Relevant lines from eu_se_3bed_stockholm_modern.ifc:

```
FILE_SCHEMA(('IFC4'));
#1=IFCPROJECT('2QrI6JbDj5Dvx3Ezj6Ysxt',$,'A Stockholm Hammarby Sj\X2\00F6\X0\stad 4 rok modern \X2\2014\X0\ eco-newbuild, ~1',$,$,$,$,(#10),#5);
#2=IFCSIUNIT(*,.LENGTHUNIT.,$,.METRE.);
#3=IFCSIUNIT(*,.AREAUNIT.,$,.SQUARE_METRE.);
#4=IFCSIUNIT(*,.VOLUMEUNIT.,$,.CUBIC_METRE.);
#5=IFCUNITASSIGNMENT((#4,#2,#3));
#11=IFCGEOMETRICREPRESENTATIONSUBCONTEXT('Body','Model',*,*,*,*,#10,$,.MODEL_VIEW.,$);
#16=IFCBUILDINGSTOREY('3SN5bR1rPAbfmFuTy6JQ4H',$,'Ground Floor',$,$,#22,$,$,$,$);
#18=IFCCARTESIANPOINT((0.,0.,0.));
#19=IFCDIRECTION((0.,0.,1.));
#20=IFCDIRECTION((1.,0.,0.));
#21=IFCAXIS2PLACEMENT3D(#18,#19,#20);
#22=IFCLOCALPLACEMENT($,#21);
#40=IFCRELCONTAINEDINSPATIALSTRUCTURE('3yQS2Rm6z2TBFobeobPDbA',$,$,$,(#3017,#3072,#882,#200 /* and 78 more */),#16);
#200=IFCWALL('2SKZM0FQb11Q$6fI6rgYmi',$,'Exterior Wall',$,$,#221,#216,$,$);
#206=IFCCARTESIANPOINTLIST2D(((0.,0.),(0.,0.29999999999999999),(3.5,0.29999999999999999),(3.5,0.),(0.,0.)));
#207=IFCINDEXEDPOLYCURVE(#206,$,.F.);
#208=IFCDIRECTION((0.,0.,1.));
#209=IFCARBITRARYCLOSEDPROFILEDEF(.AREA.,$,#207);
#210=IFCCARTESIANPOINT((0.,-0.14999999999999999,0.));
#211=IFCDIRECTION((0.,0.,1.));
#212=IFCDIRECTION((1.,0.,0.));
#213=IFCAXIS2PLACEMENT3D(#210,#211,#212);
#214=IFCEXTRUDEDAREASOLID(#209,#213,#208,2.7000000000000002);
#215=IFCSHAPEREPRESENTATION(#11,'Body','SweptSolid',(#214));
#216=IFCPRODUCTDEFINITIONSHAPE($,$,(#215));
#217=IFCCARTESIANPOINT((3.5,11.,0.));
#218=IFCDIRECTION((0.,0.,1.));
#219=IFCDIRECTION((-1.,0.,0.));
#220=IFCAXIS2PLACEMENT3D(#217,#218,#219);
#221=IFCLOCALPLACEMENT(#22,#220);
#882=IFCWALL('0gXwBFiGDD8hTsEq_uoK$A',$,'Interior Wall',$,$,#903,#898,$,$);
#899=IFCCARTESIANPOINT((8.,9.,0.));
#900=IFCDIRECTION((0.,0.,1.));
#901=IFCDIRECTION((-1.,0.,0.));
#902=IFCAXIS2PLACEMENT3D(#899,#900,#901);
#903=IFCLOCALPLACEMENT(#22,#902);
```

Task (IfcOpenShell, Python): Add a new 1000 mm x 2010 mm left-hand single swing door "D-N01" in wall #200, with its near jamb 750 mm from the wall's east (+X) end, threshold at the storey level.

```python
import numpy as np
import ifcopenshell
import ifcopenshell.api.feature
import ifcopenshell.api.geometry
import ifcopenshell.api.root
import ifcopenshell.api.spatial
import ifcopenshell.geom
import ifcopenshell.util.element
import ifcopenshell.util.placement
import ifcopenshell.util.representation
import ifcopenshell.util.shape
import ifcopenshell.util.unit

model = ifcopenshell.open("eu_se_3bed_stockholm_modern.ifc")
unit_scale = ifcopenshell.util.unit.calculate_unit_scale(model)
settings = ifcopenshell.geom.settings()


def volume(element):
    """Net volume in cubic metres, openings subtracted."""
    shape = ifcopenshell.geom.create_shape(settings, element)
    return ifcopenshell.util.shape.get_volume(shape.geometry)


wall = model.by_guid("2SKZM0FQb11Q$6fI6rgYmi")
storey = ifcopenshell.util.element.get_container(wall, ifc_class="IfcBuildingStorey")
context = ifcopenshell.util.representation.get_context(model, "Model", "Body", "MODEL_VIEW")
before = volume(wall)

width, height, from_end, sill = 1, 2.01, 0.75, 0.0  # metres

# The wall runs along its own X axis, and the end named is its -X end.
wall_shape = ifcopenshell.geom.create_shape(settings, wall)
x, y, z = ifcopenshell.util.shape.get_vertices(wall_shape.geometry).T
start = x.min() + from_end
face, thickness = float(y.min()), float(y.max() - y.min())
wall_matrix = ifcopenshell.util.placement.get_local_placement(wall.ObjectPlacement)
level = ifcopenshell.util.placement.get_local_placement(storey.ObjectPlacement)[2, 3]


def in_wall(x, y):
    """Placement at x, y metres in the wall's axes, at sill height."""
    matrix = wall_matrix.copy()
    matrix[:, 3] = wall_matrix @ np.array([x / unit_scale, y / unit_scale, 0.0, 1.0])
    matrix[2, 3] = level + sill / unit_scale
    return matrix


# Opening: a box that overshoots both wall faces by 50 mm.
opening = ifcopenshell.api.root.create_entity(model, ifc_class="IfcOpeningElement", predefined_type="OPENING")
box = ifcopenshell.api.geometry.add_wall_representation(
    model, context=context, length=width, height=height, thickness=thickness + 0.1
)
ifcopenshell.api.geometry.assign_representation(model, product=opening, representation=box)
ifcopenshell.api.geometry.edit_object_placement(model, product=opening, matrix=in_wall(start, face - 0.05), is_si=False)
ifcopenshell.api.feature.add_feature(model, feature=opening, element=wall)

door = ifcopenshell.api.root.create_entity(model, ifc_class="IfcDoor", name="D-N01", predefined_type="DOOR")
door.OverallWidth, door.OverallHeight = width / unit_scale, height / unit_scale
door.OperationType = "SINGLE_SWING_LEFT"
body = ifcopenshell.api.geometry.add_door_representation(
    model,
    context=context,
    overall_width=door.OverallWidth,
    overall_height=door.OverallHeight,
    operation_type="SINGLE_SWING_LEFT",
    lining_properties={"LiningDepth": thickness / unit_scale, "ThresholdDepth": thickness / unit_scale},
)
ifcopenshell.api.geometry.assign_representation(model, product=door, representation=body)
ifcopenshell.api.spatial.assign_container(model, products=[door], relating_structure=storey)
ifcopenshell.api.feature.add_filling(model, opening=opening, element=door)

# The lining spans the wall, so the door starts at the wall face.
ifcopenshell.api.geometry.edit_object_placement(model, product=door, matrix=in_wall(start, face), is_si=False)

after = volume(wall)

print(f"wall volume {before:.3f} -> {after:.3f} m3")

model.write("eu_se_3bed_stockholm_modern-out.ifc")
```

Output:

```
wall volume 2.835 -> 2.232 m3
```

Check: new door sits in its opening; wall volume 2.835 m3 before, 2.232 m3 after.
